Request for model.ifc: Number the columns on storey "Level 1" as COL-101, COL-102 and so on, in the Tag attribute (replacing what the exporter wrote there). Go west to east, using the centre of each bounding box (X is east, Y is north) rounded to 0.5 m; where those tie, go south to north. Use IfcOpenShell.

First a look at what the model holds.

```python
import ifcopenshell
import ifcopenshell.util.element
import ifcopenshell.util.placement

model = ifcopenshell.open("model.ifc")
print(model.schema)
storey = next(s for s in model.by_type("IfcBuildingStorey") if s.Name == "Level 1")
columns = [e for e in ifcopenshell.util.element.get_decomposition(storey) if e.is_a("IfcColumn")]
for e in sorted(columns, key=lambda e: e.id()):
    origin = ifcopenshell.util.placement.get_local_placement(e.ObjectPlacement)[:3, 3]
    print(e.id(), e.Tag, e.Name, origin.round(2) + 0.0, sep=" | ")
```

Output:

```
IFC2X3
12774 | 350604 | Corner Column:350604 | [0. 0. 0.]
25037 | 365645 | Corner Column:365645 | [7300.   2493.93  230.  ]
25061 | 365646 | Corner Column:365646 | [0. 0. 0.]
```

```python
import ifcopenshell
import ifcopenshell.geom
import ifcopenshell.util.element
import ifcopenshell.util.shape

model = ifcopenshell.open("model.ifc")
settings = ifcopenshell.geom.settings()
settings.set("use-world-coords", True)


def centre(element):
    shape = ifcopenshell.geom.create_shape(settings, element)
    return ifcopenshell.util.shape.get_bbox_centroid(shape.geometry)


storey = next(s for s in model.by_type("IfcBuildingStorey") if s.Name == "Level 1")
columns = [e for e in ifcopenshell.util.element.get_decomposition(storey) if e.is_a("IfcColumn")]

# Insertion points can sit at a corner or the storey origin, so sort by the geometry (in metres).
centres = {e: centre(e) for e in columns}
columns.sort(key=lambda e: (round(centres[e][0] / 0.5), centres[e][1]))

for i, e in enumerate(columns, start=1):
    number = f"COL-1{i:02d}"
    e.Tag = number
    print(e.id(), number)

model.write("model_updated.ifc")
```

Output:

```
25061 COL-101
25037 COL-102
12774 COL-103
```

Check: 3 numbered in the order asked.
